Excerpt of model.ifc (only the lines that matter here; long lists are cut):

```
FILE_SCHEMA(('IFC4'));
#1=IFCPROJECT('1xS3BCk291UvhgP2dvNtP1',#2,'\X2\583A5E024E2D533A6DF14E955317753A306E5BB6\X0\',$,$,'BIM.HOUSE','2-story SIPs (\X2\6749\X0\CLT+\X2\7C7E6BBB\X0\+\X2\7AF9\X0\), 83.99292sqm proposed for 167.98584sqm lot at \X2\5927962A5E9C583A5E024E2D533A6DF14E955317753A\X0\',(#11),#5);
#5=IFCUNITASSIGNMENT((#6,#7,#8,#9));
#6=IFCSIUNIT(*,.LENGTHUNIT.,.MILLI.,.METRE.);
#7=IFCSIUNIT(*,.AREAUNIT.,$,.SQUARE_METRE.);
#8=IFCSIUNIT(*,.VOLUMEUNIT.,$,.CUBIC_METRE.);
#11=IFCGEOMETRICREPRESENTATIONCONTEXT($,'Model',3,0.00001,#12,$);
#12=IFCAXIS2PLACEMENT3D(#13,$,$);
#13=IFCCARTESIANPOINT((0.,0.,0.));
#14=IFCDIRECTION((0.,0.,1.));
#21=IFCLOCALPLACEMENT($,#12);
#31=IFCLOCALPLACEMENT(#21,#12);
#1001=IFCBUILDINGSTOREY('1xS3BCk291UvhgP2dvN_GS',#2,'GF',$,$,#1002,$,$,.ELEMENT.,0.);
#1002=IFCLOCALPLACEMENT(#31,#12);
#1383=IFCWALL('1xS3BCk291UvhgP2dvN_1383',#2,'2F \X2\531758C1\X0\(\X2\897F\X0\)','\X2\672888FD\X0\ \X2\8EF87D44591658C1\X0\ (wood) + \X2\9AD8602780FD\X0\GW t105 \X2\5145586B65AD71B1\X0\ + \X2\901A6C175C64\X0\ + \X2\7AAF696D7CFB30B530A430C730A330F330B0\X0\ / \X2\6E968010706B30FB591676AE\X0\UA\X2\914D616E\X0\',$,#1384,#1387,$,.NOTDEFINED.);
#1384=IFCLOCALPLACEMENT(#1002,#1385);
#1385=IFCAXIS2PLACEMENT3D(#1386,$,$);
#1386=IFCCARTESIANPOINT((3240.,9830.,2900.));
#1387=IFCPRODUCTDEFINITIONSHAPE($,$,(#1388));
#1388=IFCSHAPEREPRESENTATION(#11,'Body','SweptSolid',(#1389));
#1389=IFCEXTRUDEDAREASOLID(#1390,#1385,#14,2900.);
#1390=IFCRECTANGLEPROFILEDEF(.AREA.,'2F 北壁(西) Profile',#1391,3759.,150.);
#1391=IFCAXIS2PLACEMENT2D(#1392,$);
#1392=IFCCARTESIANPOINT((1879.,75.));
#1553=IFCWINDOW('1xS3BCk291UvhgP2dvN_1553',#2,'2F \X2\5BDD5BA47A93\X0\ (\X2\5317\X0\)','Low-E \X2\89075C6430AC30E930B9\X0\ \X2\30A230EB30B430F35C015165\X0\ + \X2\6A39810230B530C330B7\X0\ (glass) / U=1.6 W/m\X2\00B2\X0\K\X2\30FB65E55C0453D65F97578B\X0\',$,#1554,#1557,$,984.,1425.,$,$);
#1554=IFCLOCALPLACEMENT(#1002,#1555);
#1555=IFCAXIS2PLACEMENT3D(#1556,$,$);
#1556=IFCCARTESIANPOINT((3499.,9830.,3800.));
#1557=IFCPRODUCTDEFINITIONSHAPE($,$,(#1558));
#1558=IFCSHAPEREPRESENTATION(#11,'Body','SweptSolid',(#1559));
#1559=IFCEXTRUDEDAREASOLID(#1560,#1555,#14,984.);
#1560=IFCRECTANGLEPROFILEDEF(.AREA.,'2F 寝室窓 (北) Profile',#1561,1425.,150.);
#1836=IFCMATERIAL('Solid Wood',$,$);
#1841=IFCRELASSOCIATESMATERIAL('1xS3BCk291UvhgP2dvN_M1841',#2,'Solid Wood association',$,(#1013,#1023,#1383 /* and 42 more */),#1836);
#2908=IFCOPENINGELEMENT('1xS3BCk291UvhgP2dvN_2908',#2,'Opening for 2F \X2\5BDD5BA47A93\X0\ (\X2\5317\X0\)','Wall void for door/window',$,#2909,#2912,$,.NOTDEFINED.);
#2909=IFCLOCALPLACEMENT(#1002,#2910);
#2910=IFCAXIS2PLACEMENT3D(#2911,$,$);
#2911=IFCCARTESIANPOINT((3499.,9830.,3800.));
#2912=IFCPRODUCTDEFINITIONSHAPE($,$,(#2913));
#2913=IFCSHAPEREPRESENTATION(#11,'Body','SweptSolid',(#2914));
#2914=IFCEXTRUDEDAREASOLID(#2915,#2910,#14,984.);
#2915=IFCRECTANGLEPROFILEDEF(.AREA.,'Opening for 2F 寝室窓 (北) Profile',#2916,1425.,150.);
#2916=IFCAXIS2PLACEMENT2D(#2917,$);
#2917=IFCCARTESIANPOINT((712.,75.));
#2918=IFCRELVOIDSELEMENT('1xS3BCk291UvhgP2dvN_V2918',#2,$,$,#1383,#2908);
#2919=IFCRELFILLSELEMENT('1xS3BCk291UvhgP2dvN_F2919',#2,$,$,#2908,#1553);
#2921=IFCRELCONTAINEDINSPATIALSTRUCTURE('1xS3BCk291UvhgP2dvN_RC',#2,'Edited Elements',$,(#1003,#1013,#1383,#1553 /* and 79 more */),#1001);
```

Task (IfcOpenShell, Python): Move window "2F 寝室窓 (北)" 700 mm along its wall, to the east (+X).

```python
import ifcopenshell
import ifcopenshell.api.geometry
import ifcopenshell.util.placement
import ifcopenshell.util.unit

model = ifcopenshell.open("model.ifc")
unit_scale = ifcopenshell.util.unit.calculate_unit_scale(model)

window = model.by_guid("1xS3BCk291UvhgP2dvN_1553")
opening = window.FillsVoids[0].RelatingOpeningElement
wall = opening.VoidsElements[0].RelatingBuildingElement

wall_matrix = ifcopenshell.util.placement.get_local_placement(wall.ObjectPlacement)
shift = wall_matrix[:3, 0] * 0.7 / unit_scale
before = ifcopenshell.util.placement.get_local_placement(window.ObjectPlacement)[:3, 3].copy()

# The window is not placed relative to its opening, so move both.
for product in (opening, window):
    matrix = ifcopenshell.util.placement.get_local_placement(product.ObjectPlacement)
    matrix[:3, 3] += shift
    ifcopenshell.api.geometry.edit_object_placement(model, product=product, matrix=matrix, is_si=False)

after = ifcopenshell.util.placement.get_local_placement(window.ObjectPlacement)[:3, 3]
print("window moved by", (after - before).round(3) + 0.0)

model.write("model_updated.ifc")
```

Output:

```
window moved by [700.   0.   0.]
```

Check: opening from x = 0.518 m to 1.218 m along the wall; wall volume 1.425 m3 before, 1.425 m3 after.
